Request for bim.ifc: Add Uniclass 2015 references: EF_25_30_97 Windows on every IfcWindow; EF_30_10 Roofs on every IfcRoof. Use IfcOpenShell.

First a look at what the model holds.

```python
import ifcopenshell

model = ifcopenshell.open("bim.ifc")
print(model.schema)
print("classifications:", [c.Name for c in model.by_type("IfcClassification")])
for ifc_class in ("IfcDoor", "IfcRoof", "IfcStair", "IfcWall", "IfcWindow"):
    print(ifc_class, len(model.by_type(ifc_class)))
```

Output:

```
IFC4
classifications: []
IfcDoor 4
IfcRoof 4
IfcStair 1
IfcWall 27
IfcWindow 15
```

```python
import ifcopenshell
import ifcopenshell.api.classification

model = ifcopenshell.open("bim.ifc")

system = ifcopenshell.api.classification.add_classification(model, classification="Uniclass 2015")

codes = {
    "IfcWindow": ("EF_25_30_97", "Windows"),
    "IfcRoof": ("EF_30_10", "Roofs"),
}
for ifc_class, (code, name) in codes.items():
    products = model.by_type(ifc_class)
    ifcopenshell.api.classification.add_reference(
        model, products=products, classification=system, identification=code, name=name
    )
    print(code, len(products))

model.write("bim-out.ifc")
```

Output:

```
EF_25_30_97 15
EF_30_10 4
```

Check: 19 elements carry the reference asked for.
